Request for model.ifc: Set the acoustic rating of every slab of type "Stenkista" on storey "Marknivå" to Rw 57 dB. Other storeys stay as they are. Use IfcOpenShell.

First a look at what the model holds.

```python
import ifcopenshell
import ifcopenshell.util.element

model = ifcopenshell.open("model.ifc")
print(model.schema)
storey = next(s for s in model.by_type("IfcBuildingStorey") if s.Name == "Marknivå")
slabs = [e for e in ifcopenshell.util.element.get_decomposition(storey) if e.is_a("IfcSlab")]
seen = {}
for e in slabs:
    element_type = ifcopenshell.util.element.get_type(e)
    key = (element_type.Name if element_type != e and element_type else None, ifcopenshell.util.element.get_pset(e, "Pset_SlabCommon", "AcousticRating"))
    seen[key] = seen.get(key, 0) + 1
for (name, value), count in sorted(seen.items(), key=str):
    print(count, "x", name, "|", value)
```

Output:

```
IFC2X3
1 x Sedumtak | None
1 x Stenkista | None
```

```python
import ifcopenshell
import ifcopenshell.api.pset
import ifcopenshell.util.element

model = ifcopenshell.open("model.ifc")

storey = next(s for s in model.by_type("IfcBuildingStorey") if s.Name == "Marknivå")
slabs = [e for e in ifcopenshell.util.element.get_decomposition(storey) if e.is_a("IfcSlab")]

count = 0
for e in slabs:
    element_type = ifcopenshell.util.element.get_type(e)
    if element_type in (None, e) or element_type.Name != "Stenkista":
        continue
    # add_pset returns the element's existing set when there is one.
    pset = ifcopenshell.api.pset.add_pset(model, product=e, name="Pset_SlabCommon")
    ifcopenshell.api.pset.edit_pset(model, pset=pset, properties={"AcousticRating": "Rw 57 dB"})
    count += 1

print(count, "slabs updated")

model.write("model_edited.ifc")
```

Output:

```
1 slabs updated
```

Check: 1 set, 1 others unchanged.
